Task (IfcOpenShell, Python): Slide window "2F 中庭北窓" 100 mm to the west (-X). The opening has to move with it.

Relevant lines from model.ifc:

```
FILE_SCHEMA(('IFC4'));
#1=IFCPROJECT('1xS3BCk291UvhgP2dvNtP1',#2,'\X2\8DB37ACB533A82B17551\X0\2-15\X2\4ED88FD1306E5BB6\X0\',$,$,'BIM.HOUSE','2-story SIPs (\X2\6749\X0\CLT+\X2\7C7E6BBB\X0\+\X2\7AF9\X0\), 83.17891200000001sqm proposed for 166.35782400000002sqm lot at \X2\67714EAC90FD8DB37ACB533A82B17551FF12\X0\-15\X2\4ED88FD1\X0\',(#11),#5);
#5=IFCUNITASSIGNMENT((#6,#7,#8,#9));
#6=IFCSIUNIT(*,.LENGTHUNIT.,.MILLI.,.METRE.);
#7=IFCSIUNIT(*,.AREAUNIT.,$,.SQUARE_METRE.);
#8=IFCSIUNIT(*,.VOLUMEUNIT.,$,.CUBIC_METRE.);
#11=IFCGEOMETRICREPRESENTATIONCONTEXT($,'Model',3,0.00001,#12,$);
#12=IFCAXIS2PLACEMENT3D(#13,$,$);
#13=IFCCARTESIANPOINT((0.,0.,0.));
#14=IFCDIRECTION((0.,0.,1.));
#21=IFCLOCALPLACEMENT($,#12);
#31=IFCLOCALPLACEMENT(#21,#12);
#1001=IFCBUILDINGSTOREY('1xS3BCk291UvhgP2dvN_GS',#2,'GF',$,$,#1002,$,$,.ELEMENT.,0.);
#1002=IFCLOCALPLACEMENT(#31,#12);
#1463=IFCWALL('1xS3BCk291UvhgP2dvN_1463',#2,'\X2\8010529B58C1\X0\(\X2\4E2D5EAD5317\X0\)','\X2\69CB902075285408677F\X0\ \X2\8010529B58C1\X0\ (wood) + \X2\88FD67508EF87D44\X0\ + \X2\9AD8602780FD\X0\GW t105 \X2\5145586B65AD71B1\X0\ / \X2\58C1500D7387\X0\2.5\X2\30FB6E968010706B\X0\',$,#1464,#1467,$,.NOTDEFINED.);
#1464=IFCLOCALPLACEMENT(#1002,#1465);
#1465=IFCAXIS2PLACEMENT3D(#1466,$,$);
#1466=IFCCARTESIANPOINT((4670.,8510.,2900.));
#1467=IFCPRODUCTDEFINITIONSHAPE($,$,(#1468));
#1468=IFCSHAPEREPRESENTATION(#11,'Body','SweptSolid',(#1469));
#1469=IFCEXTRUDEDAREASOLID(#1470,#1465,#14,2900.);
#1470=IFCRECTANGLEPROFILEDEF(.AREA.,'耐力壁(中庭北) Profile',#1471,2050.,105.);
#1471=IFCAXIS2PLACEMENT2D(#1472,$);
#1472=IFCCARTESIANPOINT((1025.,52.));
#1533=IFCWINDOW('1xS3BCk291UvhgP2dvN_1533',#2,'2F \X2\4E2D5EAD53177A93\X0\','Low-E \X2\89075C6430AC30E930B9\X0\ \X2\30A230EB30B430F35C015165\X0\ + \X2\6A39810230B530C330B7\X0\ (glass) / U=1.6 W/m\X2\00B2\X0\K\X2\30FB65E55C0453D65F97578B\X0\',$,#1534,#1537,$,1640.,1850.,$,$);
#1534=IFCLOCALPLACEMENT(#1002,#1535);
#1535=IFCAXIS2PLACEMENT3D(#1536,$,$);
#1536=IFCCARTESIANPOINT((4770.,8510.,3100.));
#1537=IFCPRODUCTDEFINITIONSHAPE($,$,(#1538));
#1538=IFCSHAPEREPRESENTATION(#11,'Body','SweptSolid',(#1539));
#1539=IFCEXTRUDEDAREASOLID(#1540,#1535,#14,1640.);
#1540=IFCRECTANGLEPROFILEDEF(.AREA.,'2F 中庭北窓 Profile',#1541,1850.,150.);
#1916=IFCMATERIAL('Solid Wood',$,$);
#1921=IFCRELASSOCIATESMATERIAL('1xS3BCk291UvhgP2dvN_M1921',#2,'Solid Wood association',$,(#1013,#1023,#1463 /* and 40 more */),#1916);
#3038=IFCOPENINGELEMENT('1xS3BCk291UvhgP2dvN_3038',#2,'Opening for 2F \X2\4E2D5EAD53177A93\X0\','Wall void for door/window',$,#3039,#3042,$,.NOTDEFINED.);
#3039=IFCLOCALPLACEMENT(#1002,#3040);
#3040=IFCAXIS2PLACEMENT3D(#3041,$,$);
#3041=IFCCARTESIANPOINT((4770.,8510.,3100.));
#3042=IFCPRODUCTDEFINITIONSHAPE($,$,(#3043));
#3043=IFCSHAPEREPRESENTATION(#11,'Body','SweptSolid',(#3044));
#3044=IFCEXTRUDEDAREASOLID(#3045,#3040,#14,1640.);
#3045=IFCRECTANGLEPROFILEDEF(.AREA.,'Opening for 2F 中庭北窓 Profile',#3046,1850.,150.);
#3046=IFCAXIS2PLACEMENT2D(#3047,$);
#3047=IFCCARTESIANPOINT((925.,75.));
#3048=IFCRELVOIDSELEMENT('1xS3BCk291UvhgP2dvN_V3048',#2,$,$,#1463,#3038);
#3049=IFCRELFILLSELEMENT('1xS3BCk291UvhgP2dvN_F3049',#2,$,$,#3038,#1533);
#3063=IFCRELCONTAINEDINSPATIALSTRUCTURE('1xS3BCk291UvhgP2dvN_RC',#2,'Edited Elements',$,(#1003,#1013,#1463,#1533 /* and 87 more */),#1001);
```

```python
import ifcopenshell
import ifcopenshell.api.geometry
import ifcopenshell.util.placement

model = ifcopenshell.open("model.ifc")

window = model.by_guid("1xS3BCk291UvhgP2dvN_1533")
opening = window.FillsVoids[0].RelatingOpeningElement
wall = opening.VoidsElements[0].RelatingBuildingElement

wall_matrix = ifcopenshell.util.placement.get_local_placement(wall.ObjectPlacement)
shift = wall_matrix[:3, 0] * -100.0
before = ifcopenshell.util.placement.get_local_placement(window.ObjectPlacement)[:3, 3].copy()

# The window is not placed relative to its opening, so move both.
for product in (opening, window):
    matrix = ifcopenshell.util.placement.get_local_placement(product.ObjectPlacement)
    matrix[:3, 3] += shift
    ifcopenshell.api.geometry.edit_object_placement(model, product=product, matrix=matrix, is_si=False)

after = ifcopenshell.util.placement.get_local_placement(window.ObjectPlacement)[:3, 3]
print("window moved by", (after - before).round(3) + 0.0)

model.write("model_updated.ifc")
```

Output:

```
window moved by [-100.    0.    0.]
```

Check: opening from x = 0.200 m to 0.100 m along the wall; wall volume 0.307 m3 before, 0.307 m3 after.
